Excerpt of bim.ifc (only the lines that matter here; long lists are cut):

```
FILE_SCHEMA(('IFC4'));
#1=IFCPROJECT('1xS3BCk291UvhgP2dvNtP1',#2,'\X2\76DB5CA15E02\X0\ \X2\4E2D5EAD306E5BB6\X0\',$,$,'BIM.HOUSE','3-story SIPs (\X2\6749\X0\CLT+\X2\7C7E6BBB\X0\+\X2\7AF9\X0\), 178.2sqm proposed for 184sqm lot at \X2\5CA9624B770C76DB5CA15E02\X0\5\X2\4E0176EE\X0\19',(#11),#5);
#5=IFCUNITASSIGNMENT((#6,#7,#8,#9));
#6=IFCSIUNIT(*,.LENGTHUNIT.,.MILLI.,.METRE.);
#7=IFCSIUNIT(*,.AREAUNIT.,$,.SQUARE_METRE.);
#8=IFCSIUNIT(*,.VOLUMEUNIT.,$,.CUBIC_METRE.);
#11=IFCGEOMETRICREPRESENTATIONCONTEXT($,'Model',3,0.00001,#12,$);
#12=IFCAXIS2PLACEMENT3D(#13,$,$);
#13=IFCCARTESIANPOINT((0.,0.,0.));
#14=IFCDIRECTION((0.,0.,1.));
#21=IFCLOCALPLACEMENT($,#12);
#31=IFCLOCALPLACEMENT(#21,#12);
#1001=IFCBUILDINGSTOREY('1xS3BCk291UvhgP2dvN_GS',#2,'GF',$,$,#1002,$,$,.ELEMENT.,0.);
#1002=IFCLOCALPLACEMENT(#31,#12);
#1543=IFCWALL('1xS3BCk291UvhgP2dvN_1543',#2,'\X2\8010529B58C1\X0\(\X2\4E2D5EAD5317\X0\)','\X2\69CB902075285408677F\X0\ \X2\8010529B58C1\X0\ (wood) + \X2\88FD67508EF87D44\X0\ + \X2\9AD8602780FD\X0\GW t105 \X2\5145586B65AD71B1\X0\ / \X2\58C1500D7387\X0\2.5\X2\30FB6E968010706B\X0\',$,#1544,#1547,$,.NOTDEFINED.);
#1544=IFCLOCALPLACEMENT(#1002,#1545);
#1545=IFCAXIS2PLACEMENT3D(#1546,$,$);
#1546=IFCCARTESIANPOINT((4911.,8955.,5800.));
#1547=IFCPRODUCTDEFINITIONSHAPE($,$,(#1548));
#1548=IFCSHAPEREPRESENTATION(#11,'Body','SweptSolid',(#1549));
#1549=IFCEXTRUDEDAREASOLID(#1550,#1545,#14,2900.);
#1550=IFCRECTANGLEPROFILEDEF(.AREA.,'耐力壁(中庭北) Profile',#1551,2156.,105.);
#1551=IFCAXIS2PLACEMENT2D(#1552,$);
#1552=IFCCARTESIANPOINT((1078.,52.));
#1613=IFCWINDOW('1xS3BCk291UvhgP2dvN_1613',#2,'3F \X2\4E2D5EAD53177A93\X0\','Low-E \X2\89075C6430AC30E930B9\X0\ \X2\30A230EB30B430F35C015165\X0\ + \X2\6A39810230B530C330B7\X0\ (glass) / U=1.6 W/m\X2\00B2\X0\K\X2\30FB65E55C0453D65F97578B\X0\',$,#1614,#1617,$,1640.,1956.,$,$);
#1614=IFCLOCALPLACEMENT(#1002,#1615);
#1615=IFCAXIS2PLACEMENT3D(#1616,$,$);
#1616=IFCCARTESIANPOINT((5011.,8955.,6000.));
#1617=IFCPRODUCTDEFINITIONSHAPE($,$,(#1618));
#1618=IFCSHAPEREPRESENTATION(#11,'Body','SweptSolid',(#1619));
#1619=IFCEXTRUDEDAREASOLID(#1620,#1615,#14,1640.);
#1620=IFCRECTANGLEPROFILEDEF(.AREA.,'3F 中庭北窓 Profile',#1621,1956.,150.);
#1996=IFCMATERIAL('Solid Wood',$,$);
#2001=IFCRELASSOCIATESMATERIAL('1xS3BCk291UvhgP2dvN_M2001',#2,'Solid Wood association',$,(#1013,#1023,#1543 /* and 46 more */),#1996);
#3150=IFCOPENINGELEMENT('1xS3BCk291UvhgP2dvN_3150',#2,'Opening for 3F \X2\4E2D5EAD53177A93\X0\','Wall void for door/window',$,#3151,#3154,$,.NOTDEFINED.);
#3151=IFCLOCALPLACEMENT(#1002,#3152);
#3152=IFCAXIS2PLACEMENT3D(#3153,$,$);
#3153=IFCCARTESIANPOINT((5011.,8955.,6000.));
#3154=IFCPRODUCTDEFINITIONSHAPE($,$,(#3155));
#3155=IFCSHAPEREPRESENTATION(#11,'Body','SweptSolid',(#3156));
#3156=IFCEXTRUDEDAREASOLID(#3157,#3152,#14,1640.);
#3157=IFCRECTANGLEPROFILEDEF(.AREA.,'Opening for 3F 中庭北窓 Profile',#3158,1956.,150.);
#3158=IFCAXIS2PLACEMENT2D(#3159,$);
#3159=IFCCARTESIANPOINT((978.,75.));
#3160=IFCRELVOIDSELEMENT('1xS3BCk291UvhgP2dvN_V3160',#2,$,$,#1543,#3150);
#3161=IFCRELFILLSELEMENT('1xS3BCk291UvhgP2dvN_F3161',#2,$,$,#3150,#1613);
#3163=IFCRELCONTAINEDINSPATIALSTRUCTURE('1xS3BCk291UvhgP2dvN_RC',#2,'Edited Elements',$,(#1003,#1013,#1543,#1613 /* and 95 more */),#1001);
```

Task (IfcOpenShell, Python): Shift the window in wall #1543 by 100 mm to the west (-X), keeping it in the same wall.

```python
import ifcopenshell
import ifcopenshell.api.geometry
import ifcopenshell.util.placement

model = ifcopenshell.open("bim.ifc")

window = model.by_id(1613)
opening = window.FillsVoids[0].RelatingOpeningElement
wall = opening.VoidsElements[0].RelatingBuildingElement

wall_matrix = ifcopenshell.util.placement.get_local_placement(wall.ObjectPlacement)
shift = wall_matrix[:3, 0] * -100.0
before = ifcopenshell.util.placement.get_local_placement(window.ObjectPlacement)[:3, 3].copy()

# The window is not placed relative to its opening, so move both.
for product in (opening, window):
    matrix = ifcopenshell.util.placement.get_local_placement(product.ObjectPlacement)
    matrix[:3, 3] += shift
    ifcopenshell.api.geometry.edit_object_placement(model, product=product, matrix=matrix, is_si=False)

after = ifcopenshell.util.placement.get_local_placement(window.ObjectPlacement)[:3, 3]
print("window moved by", (after - before).round(3) + 0.0)

model.write("bim_updated.ifc")
```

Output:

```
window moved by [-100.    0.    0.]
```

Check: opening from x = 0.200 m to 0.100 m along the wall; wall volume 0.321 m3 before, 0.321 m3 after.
